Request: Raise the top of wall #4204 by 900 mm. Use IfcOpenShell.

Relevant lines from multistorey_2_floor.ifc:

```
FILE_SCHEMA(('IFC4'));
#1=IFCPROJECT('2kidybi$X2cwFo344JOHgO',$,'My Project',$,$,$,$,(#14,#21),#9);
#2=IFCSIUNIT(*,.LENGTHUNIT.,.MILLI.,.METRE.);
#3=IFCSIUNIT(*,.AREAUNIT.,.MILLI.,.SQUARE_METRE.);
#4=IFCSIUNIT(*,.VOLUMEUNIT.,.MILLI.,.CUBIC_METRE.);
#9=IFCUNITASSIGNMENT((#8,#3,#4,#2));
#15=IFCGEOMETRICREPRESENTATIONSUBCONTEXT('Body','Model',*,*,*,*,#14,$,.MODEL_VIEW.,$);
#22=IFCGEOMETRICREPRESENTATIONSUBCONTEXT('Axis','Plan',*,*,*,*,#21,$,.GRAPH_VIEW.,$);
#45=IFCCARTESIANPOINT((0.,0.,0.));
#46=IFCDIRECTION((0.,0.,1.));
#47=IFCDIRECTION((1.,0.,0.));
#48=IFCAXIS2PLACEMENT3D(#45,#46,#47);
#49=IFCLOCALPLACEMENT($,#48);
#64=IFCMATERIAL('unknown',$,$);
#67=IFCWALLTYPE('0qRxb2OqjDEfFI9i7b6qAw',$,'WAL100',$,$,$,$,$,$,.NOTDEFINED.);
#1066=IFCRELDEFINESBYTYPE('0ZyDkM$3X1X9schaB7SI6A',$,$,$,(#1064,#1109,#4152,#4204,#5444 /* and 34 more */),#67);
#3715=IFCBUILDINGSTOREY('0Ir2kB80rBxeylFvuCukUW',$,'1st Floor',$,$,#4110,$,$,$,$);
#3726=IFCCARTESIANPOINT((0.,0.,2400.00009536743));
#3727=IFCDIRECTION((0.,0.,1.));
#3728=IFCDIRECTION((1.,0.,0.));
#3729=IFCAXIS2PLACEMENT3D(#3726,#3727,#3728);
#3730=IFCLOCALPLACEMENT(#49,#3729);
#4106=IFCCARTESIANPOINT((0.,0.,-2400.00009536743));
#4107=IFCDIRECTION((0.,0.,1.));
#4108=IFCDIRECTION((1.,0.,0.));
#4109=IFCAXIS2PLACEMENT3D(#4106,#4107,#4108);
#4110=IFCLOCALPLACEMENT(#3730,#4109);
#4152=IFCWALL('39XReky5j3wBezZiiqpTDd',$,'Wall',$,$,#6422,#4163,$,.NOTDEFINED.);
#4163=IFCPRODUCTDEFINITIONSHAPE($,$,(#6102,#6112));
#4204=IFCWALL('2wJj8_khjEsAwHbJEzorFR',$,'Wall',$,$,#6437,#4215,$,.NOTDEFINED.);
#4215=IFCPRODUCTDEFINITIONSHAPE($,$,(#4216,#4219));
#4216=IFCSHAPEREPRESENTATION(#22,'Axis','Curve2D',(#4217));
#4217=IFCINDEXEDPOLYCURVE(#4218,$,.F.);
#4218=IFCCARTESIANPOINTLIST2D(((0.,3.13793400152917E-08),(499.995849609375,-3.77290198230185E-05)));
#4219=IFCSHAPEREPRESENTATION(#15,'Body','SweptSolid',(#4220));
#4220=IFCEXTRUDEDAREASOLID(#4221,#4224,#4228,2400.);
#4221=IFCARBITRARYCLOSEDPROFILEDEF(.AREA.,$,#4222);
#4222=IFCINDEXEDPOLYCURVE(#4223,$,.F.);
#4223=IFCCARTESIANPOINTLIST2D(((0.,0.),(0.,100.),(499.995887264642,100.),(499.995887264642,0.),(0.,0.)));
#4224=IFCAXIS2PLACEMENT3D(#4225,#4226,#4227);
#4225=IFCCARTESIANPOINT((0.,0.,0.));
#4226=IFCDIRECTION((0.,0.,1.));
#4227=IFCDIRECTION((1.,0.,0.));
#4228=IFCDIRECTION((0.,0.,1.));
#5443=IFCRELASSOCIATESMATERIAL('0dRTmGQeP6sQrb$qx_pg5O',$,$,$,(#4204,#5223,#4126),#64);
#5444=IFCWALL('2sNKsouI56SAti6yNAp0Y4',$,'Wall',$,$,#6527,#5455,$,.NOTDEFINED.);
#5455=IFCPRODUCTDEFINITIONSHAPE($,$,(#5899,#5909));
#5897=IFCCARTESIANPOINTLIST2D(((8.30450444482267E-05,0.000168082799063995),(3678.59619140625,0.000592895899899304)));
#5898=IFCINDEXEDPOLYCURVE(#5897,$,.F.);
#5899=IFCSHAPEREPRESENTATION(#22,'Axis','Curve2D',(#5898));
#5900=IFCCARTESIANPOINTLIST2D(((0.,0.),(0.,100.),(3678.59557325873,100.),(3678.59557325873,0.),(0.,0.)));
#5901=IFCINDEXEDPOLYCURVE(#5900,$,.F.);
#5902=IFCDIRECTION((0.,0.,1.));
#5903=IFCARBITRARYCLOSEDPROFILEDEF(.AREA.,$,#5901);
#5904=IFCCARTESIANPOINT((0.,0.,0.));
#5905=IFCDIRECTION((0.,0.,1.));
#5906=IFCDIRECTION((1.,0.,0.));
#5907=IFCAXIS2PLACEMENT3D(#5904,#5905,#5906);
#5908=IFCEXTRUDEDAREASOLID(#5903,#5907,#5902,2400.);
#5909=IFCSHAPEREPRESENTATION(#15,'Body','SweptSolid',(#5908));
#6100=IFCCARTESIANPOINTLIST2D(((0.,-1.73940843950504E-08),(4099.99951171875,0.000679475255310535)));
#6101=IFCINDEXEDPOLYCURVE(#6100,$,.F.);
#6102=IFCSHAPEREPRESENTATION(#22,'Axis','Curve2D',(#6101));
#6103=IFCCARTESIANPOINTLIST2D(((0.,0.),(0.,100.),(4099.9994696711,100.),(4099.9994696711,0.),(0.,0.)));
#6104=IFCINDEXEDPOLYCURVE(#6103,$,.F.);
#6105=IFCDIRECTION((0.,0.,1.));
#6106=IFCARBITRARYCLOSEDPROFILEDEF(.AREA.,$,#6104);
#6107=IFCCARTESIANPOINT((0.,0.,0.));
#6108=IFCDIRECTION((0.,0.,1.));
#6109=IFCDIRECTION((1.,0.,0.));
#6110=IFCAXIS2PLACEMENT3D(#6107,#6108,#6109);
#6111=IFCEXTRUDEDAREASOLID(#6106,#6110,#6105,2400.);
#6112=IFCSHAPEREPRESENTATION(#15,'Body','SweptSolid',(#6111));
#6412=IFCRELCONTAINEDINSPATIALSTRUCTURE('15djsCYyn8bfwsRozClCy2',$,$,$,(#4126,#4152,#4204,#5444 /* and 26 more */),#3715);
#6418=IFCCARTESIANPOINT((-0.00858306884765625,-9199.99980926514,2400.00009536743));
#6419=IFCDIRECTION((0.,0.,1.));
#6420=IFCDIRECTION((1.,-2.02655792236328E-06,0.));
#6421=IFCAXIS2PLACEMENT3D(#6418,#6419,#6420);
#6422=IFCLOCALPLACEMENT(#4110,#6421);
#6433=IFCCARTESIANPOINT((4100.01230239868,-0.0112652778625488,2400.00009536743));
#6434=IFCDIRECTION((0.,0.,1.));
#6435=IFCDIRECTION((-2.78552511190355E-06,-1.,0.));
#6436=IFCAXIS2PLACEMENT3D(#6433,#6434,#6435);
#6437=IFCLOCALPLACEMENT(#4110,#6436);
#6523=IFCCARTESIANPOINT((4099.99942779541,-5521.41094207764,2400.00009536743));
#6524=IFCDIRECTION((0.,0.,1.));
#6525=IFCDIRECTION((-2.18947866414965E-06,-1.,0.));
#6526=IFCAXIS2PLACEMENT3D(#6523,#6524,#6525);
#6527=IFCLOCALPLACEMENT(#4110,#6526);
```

```python
import ifcopenshell
import ifcopenshell.geom
import ifcopenshell.util.representation
import ifcopenshell.util.shape
import ifcopenshell.util.unit

model = ifcopenshell.open("multistorey_2_floor.ifc")
unit_scale = ifcopenshell.util.unit.calculate_unit_scale(model)
settings = ifcopenshell.geom.settings()


def volume(element):
    """Net volume in cubic metres, openings subtracted."""
    shape = ifcopenshell.geom.create_shape(settings, element)
    return ifcopenshell.util.shape.get_volume(shape.geometry)


wall = model.by_id(4204)
before = volume(wall)

body = ifcopenshell.util.representation.get_representation(wall, "Model", "Body")
solid = body.Items[0]
old_height = solid.Depth
solid.Depth += 0.9 / unit_scale
after = volume(wall)

print(f"height {old_height:g} -> {solid.Depth:g}, volume {before:.3f} -> {after:.3f} m3")

model.write("multistorey_2_floor_v2.ifc")
```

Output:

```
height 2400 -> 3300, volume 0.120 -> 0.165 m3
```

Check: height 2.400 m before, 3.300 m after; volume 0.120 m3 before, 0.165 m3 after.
